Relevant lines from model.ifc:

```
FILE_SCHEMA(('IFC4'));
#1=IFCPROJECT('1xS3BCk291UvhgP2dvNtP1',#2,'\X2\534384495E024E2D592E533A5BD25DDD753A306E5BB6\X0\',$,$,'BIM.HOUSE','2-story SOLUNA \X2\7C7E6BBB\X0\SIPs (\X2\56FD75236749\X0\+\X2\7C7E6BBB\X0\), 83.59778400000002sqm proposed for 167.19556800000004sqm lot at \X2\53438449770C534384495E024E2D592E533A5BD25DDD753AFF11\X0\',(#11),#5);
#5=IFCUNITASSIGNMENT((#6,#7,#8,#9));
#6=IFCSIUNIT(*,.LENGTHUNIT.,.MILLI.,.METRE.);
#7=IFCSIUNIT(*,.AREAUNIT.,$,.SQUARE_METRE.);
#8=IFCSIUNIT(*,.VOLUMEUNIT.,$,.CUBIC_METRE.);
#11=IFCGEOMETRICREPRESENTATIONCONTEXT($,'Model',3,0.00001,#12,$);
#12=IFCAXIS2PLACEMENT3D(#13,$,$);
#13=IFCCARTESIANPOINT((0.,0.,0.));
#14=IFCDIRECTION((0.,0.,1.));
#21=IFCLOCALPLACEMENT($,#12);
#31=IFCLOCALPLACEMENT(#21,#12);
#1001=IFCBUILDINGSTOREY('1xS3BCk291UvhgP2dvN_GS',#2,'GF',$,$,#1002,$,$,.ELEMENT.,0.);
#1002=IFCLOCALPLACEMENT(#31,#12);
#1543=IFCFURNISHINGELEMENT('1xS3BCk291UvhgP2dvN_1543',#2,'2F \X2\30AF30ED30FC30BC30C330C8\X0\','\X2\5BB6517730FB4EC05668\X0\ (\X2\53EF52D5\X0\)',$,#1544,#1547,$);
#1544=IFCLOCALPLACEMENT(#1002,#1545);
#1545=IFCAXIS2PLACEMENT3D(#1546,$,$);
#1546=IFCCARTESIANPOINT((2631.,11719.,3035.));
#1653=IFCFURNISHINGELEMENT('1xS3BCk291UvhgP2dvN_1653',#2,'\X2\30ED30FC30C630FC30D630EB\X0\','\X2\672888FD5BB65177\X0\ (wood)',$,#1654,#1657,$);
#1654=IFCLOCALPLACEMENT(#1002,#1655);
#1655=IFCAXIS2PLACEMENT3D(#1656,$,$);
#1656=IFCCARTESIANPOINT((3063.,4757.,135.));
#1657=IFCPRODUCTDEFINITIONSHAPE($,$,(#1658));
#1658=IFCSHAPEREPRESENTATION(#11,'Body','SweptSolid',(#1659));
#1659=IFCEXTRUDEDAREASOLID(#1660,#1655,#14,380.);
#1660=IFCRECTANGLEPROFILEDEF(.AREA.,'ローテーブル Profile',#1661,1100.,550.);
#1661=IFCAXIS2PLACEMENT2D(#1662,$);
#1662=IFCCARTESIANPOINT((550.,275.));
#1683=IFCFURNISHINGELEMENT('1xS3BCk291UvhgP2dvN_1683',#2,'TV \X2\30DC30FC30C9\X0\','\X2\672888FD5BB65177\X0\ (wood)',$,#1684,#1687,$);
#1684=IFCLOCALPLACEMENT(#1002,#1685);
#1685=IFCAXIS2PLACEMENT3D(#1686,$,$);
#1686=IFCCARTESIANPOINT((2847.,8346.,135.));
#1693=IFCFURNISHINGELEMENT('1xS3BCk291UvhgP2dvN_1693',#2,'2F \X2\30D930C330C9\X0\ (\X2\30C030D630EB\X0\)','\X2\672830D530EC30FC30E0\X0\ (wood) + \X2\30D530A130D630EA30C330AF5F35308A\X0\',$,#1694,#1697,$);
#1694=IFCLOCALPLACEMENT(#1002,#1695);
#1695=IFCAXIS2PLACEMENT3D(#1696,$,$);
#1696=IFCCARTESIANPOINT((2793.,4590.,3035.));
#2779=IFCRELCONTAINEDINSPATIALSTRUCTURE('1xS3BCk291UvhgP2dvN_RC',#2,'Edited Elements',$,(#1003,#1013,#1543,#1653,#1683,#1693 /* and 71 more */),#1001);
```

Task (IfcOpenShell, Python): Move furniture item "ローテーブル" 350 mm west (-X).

```python
import ifcopenshell
import ifcopenshell.api.geometry
import ifcopenshell.util.placement

model = ifcopenshell.open("model.ifc")

item = model.by_guid("1xS3BCk291UvhgP2dvN_1653")
matrix = ifcopenshell.util.placement.get_local_placement(item.ObjectPlacement)
matrix[0, 3] -= 350.0
ifcopenshell.api.geometry.edit_object_placement(model, product=item, matrix=matrix, is_si=False)

print(ifcopenshell.util.placement.get_local_placement(item.ObjectPlacement).round(3) + 0.0)

model.write("model-out.ifc")
```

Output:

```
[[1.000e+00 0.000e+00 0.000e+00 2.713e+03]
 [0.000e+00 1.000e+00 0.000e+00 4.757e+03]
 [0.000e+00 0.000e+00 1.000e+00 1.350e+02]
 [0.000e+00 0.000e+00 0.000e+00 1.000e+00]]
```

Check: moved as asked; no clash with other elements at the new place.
